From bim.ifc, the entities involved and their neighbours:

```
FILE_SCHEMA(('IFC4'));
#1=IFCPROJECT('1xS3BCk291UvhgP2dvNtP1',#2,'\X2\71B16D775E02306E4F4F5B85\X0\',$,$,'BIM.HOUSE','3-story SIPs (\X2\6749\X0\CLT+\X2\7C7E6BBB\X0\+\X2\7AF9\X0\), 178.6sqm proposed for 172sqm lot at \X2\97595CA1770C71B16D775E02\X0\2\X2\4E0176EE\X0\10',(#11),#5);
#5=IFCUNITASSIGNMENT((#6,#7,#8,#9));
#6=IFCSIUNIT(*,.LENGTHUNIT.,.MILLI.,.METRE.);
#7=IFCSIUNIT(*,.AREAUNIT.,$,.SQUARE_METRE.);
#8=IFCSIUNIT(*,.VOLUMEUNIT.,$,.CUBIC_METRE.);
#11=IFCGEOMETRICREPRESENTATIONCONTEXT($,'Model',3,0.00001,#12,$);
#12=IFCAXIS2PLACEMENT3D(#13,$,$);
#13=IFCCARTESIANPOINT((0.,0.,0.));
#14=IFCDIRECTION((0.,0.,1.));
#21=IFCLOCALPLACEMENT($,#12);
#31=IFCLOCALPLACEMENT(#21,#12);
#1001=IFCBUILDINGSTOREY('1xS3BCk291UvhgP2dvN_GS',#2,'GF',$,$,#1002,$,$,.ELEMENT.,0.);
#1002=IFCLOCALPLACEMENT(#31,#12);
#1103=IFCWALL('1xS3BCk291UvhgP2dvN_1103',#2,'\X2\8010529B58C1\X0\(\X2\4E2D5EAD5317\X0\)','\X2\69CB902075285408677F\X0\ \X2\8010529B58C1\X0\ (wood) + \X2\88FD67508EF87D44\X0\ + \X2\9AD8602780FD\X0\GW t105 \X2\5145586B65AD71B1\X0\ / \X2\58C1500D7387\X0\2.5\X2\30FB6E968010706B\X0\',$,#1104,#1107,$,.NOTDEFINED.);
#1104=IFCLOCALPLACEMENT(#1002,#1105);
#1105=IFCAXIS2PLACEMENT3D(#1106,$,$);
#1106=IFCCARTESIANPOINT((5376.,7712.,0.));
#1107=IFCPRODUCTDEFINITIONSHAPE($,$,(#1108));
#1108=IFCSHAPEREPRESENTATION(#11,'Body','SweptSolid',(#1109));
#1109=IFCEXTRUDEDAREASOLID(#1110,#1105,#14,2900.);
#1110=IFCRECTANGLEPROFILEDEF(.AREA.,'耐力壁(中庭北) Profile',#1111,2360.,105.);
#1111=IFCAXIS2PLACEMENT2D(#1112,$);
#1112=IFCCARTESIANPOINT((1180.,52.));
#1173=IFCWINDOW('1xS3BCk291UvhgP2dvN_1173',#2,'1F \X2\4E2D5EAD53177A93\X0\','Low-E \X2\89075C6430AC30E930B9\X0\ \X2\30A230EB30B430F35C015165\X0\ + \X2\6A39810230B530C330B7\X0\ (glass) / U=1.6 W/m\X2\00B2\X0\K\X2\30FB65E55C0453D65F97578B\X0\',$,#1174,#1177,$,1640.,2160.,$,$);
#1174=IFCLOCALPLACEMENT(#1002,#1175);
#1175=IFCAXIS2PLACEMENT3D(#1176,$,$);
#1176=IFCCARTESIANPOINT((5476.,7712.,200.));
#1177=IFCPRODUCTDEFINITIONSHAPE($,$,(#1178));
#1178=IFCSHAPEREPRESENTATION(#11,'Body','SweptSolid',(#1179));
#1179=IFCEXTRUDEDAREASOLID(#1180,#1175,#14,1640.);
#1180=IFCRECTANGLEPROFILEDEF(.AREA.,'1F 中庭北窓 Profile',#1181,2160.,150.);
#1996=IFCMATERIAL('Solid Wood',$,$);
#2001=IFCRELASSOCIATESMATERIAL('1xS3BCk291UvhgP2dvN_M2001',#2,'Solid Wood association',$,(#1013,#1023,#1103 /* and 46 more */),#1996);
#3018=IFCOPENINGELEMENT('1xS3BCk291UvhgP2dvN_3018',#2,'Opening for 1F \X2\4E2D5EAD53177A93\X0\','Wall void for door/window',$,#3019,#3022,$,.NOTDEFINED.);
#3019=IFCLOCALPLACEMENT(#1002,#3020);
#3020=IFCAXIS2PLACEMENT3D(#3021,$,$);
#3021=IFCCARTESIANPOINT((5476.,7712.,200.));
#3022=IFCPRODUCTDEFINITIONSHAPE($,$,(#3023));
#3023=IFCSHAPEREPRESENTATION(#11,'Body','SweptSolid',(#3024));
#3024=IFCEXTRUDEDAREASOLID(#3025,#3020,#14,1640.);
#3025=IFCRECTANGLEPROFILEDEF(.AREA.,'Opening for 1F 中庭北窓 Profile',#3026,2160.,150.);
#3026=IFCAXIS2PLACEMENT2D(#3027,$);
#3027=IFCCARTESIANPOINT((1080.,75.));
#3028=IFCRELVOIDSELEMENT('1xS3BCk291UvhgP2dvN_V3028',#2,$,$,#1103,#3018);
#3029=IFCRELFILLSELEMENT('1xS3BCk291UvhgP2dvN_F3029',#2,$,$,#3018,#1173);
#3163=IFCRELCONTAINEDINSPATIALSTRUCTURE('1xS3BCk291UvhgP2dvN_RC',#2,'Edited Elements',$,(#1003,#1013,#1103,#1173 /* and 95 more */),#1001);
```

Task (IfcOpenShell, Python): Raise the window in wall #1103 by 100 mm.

```python
import numpy as np
import ifcopenshell
import ifcopenshell.api.geometry
import ifcopenshell.util.placement
import ifcopenshell.util.unit

model = ifcopenshell.open("bim.ifc")
unit_scale = ifcopenshell.util.unit.calculate_unit_scale(model)

window = model.by_guid("1xS3BCk291UvhgP2dvN_1173")
opening = window.FillsVoids[0].RelatingOpeningElement
dz = 0.1 / unit_scale

shift = np.array([0.0, 0.0, dz])
# The window is not placed relative to its opening, so move both.
for product in (opening, window):
    matrix = ifcopenshell.util.placement.get_local_placement(product.ObjectPlacement)
    matrix[:3, 3] += shift
    ifcopenshell.api.geometry.edit_object_placement(model, product=product, matrix=matrix, is_si=False)

print(f"moved by {dz * unit_scale:+.3f} m")

model.write("bim_updated.ifc")
```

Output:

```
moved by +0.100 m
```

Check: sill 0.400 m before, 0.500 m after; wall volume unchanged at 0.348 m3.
